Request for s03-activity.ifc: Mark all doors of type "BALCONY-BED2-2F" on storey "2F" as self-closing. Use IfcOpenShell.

First a look at what the model holds.

```python
import ifcopenshell
import ifcopenshell.util.element

model = ifcopenshell.open("s03-activity.ifc")
print(model.schema)
storey = next(s for s in model.by_type("IfcBuildingStorey") if s.Name == "2F")
doors = [e for e in ifcopenshell.util.element.get_decomposition(storey) if e.is_a("IfcDoor")]
seen = {}
for e in doors:
    element_type = ifcopenshell.util.element.get_type(e)
    key = (element_type.Name if element_type != e and element_type else None, ifcopenshell.util.element.get_pset(e, "Pset_DoorCommon", "SelfClosing"))
    seen[key] = seen.get(key, 0) + 1
for (name, value), count in sorted(seen.items(), key=str):
    print(count, "x", name, "|", value)
```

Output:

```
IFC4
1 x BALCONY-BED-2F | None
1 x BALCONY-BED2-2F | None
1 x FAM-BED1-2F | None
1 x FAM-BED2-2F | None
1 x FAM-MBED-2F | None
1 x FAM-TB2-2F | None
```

```python
import ifcopenshell
import ifcopenshell.api.pset
import ifcopenshell.util.element

model = ifcopenshell.open("s03-activity.ifc")

storey = next(s for s in model.by_type("IfcBuildingStorey") if s.Name == "2F")
doors = [e for e in ifcopenshell.util.element.get_decomposition(storey) if e.is_a("IfcDoor")]

count = 0
for e in doors:
    element_type = ifcopenshell.util.element.get_type(e)
    if element_type in (None, e) or element_type.Name != "BALCONY-BED2-2F":
        continue
    # add_pset returns the element's existing set when there is one.
    pset = ifcopenshell.api.pset.add_pset(model, product=e, name="Pset_DoorCommon")
    ifcopenshell.api.pset.edit_pset(model, pset=pset, properties={"SelfClosing": True})
    count += 1

print(count, "doors updated")

model.write("s03-activity-out.ifc")
```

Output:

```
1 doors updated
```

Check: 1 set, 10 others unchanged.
